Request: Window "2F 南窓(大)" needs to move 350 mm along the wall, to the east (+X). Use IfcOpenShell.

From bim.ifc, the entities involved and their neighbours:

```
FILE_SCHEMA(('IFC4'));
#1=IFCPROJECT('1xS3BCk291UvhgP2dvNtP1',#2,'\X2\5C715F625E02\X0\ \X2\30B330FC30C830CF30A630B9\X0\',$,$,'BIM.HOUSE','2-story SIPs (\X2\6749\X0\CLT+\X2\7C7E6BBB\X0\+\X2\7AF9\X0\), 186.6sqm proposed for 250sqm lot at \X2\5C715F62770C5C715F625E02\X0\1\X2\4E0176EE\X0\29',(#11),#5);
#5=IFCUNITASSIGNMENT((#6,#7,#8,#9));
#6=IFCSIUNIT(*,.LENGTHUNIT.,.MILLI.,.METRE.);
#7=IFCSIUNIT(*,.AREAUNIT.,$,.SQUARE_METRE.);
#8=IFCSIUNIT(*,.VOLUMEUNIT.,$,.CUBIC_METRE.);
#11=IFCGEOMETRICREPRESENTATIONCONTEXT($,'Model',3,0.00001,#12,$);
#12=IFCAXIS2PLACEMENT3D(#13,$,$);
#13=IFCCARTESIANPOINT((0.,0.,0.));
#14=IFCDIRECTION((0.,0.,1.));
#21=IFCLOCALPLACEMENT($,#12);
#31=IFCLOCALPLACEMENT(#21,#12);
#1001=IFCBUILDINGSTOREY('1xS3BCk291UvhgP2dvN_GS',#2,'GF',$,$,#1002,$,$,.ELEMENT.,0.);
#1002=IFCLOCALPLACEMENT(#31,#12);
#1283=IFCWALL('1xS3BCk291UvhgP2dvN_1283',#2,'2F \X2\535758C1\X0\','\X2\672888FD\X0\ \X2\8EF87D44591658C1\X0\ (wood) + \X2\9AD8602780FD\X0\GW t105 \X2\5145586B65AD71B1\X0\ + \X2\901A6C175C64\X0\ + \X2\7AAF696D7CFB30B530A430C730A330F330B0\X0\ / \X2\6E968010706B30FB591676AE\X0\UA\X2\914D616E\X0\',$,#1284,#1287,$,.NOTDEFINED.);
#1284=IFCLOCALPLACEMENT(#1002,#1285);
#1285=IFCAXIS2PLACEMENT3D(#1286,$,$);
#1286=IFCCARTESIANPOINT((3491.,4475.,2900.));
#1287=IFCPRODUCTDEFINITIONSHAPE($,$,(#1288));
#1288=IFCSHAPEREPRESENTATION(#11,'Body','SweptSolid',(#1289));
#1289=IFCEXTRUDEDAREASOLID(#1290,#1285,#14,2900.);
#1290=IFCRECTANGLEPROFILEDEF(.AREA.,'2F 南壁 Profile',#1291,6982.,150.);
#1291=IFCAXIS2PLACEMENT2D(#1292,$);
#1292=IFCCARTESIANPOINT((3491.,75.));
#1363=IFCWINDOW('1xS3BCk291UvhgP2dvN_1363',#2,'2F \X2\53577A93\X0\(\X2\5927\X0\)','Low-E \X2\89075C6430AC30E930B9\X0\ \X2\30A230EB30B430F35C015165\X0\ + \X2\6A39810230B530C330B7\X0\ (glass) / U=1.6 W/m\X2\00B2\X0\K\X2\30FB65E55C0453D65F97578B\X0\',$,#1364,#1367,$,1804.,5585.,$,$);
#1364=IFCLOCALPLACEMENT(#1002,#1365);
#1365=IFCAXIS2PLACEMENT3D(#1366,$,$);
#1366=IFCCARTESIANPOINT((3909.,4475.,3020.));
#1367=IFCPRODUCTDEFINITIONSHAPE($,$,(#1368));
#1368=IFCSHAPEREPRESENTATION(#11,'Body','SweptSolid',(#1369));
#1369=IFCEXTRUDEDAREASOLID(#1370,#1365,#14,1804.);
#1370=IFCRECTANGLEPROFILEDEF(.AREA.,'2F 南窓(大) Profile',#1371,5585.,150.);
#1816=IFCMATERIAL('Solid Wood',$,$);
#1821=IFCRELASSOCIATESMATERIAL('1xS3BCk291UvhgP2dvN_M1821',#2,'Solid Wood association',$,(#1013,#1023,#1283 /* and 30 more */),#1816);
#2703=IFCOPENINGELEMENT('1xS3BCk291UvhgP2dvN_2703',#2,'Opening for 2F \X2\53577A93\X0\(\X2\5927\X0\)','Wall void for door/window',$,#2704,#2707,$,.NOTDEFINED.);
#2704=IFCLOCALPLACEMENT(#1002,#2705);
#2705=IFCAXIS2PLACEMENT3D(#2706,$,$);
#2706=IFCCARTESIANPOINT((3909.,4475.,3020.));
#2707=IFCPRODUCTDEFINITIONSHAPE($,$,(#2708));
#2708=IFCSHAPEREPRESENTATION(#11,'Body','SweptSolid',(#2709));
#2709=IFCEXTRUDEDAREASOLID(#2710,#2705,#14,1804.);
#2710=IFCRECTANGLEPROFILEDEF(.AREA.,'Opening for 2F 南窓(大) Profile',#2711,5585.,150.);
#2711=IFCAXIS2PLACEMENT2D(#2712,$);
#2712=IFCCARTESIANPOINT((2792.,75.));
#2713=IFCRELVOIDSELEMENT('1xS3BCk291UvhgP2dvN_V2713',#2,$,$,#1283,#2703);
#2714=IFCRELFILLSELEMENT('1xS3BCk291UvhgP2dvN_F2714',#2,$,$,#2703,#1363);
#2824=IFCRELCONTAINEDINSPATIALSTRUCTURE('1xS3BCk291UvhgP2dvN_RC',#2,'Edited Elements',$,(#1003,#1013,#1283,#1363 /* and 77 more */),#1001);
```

```python
import ifcopenshell
import ifcopenshell.api.geometry
import ifcopenshell.util.placement

model = ifcopenshell.open("bim.ifc")

window = model.by_guid("1xS3BCk291UvhgP2dvN_1363")
opening = window.FillsVoids[0].RelatingOpeningElement
wall = opening.VoidsElements[0].RelatingBuildingElement

wall_matrix = ifcopenshell.util.placement.get_local_placement(wall.ObjectPlacement)
shift = wall_matrix[:3, 0] * 350.0
before = ifcopenshell.util.placement.get_local_placement(window.ObjectPlacement)[:3, 3].copy()

# The window is not placed relative to its opening, so move both.
for product in (opening, window):
    matrix = ifcopenshell.util.placement.get_local_placement(product.ObjectPlacement)
    matrix[:3, 3] += shift
    ifcopenshell.api.geometry.edit_object_placement(model, product=product, matrix=matrix, is_si=False)

after = ifcopenshell.util.placement.get_local_placement(window.ObjectPlacement)[:3, 3]
print("window moved by", (after - before).round(3) + 0.0)

model.write("bim_edited.ifc")
```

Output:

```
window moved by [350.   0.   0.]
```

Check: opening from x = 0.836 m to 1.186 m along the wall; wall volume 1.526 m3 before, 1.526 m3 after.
